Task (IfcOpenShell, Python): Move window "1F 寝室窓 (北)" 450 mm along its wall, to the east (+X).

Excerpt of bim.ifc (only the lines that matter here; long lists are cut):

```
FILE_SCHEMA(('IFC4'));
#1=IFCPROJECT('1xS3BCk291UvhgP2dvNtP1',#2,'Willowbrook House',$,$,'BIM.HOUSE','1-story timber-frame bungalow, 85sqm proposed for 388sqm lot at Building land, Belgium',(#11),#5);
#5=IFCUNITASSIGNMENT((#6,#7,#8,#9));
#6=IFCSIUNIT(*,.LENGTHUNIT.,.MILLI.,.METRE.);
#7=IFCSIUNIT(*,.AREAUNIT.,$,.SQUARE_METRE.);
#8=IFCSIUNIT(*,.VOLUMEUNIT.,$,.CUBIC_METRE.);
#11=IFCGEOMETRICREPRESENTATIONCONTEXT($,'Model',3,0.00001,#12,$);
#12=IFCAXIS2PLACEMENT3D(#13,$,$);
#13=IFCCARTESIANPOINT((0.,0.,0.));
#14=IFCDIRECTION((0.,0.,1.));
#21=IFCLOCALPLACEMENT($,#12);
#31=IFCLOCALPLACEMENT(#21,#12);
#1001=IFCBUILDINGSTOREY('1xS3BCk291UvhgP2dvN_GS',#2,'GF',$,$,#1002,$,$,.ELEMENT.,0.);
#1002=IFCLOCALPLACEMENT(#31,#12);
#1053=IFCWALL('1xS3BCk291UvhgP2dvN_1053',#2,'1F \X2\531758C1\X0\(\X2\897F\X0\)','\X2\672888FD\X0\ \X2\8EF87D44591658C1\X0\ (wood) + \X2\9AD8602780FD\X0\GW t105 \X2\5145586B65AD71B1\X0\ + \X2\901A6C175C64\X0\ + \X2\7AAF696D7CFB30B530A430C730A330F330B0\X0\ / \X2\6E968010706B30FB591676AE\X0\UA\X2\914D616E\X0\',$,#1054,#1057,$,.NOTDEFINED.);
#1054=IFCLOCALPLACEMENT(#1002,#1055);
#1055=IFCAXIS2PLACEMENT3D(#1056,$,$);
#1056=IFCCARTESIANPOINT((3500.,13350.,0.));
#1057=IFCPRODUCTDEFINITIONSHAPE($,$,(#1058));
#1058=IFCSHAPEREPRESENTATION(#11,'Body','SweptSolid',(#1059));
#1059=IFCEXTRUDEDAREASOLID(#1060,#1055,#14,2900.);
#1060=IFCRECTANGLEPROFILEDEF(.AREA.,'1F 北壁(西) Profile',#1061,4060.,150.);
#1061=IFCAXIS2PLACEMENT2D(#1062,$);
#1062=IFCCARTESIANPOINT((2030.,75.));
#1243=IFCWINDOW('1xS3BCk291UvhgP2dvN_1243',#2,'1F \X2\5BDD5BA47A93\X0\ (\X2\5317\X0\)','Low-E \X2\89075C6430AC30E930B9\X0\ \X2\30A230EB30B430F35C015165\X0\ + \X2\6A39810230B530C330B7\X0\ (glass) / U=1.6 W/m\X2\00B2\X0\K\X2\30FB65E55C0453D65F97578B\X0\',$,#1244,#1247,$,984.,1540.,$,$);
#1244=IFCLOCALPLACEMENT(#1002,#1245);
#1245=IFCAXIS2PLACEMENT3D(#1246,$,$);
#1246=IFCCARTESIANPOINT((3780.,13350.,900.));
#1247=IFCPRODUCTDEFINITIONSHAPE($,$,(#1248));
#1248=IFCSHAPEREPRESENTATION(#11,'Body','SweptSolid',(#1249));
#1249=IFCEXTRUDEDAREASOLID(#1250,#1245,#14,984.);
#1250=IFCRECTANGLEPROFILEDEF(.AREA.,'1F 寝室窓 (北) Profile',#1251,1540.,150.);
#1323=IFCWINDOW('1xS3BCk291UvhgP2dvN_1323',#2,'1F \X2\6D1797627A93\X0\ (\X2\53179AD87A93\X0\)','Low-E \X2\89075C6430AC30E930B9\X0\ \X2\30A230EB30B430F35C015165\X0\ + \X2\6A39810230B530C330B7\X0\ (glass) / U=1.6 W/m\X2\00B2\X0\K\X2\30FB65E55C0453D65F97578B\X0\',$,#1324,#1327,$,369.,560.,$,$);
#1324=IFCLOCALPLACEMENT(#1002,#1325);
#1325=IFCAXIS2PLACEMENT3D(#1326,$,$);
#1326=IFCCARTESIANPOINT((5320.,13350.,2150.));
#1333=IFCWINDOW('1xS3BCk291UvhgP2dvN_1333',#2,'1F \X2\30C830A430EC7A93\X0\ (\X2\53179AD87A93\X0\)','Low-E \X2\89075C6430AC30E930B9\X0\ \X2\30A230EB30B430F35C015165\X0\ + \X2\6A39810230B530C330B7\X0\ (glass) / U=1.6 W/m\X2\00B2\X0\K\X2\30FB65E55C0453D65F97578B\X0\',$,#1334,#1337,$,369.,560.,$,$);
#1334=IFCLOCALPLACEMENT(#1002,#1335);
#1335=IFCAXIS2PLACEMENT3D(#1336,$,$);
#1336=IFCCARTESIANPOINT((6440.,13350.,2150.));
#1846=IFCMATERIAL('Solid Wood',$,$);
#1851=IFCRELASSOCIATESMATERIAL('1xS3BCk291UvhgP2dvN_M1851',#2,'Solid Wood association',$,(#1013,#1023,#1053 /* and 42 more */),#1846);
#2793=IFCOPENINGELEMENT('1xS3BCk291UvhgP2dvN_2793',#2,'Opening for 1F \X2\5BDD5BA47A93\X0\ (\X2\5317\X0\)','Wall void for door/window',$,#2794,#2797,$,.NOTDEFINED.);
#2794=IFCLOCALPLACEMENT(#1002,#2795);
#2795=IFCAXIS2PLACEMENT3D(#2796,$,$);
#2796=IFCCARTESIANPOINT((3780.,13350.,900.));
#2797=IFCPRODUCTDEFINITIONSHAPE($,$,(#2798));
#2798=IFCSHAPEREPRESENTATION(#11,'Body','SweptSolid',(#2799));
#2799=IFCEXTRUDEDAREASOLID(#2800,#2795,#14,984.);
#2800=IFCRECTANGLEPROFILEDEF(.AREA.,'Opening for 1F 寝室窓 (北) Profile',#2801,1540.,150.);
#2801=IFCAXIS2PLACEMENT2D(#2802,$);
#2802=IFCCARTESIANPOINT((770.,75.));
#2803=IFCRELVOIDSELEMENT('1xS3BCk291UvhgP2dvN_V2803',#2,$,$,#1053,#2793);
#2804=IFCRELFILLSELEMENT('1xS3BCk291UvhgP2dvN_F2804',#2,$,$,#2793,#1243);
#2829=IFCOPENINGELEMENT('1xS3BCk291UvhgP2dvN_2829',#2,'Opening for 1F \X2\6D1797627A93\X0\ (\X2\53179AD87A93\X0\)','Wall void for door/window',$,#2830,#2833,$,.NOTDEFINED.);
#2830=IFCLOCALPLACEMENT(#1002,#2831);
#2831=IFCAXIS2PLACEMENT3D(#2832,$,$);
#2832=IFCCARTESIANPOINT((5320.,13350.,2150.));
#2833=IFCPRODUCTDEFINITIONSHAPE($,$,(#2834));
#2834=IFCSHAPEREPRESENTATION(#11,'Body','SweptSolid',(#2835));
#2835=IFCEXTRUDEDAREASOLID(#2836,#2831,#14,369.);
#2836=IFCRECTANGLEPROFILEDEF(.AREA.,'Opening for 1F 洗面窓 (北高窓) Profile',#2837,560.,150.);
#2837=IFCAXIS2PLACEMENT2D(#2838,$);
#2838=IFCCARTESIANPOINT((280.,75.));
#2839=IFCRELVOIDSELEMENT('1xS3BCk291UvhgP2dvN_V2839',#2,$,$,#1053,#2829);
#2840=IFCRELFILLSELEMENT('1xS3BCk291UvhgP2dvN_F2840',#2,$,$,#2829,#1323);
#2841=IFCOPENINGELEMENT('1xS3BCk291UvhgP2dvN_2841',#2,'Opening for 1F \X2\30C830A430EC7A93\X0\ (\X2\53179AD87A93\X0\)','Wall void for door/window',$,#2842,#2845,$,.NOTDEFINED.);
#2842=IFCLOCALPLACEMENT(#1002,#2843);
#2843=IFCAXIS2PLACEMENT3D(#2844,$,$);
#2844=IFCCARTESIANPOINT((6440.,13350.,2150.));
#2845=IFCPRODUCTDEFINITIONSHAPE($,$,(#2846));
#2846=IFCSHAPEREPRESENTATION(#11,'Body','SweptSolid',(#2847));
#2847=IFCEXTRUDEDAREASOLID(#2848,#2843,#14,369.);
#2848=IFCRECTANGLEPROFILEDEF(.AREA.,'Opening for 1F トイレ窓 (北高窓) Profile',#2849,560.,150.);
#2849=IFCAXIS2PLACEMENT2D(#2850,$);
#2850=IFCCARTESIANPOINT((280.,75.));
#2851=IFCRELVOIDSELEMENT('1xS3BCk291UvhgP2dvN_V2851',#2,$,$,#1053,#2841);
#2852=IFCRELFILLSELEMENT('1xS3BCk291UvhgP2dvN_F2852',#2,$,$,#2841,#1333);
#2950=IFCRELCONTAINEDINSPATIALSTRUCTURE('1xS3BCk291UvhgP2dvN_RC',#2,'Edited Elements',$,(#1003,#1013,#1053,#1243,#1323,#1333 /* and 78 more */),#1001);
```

```python
import ifcopenshell
import ifcopenshell.api.geometry
import ifcopenshell.util.placement
import ifcopenshell.util.unit

model = ifcopenshell.open("bim.ifc")
unit_scale = ifcopenshell.util.unit.calculate_unit_scale(model)

window = model.by_guid("1xS3BCk291UvhgP2dvN_1243")
opening = window.FillsVoids[0].RelatingOpeningElement
wall = opening.VoidsElements[0].RelatingBuildingElement

wall_matrix = ifcopenshell.util.placement.get_local_placement(wall.ObjectPlacement)
shift = wall_matrix[:3, 0] * 0.45 / unit_scale
before = ifcopenshell.util.placement.get_local_placement(window.ObjectPlacement)[:3, 3].copy()

# The window is not placed relative to its opening, so move both.
for product in (opening, window):
    matrix = ifcopenshell.util.placement.get_local_placement(product.ObjectPlacement)
    matrix[:3, 3] += shift
    ifcopenshell.api.geometry.edit_object_placement(model, product=product, matrix=matrix, is_si=False)

after = ifcopenshell.util.placement.get_local_placement(window.ObjectPlacement)[:3, 3]
print("window moved by", (after - before).round(3) + 0.0)

model.write("bim_updated.ifc")
```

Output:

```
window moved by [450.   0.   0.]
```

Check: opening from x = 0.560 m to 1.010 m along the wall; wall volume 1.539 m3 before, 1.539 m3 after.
